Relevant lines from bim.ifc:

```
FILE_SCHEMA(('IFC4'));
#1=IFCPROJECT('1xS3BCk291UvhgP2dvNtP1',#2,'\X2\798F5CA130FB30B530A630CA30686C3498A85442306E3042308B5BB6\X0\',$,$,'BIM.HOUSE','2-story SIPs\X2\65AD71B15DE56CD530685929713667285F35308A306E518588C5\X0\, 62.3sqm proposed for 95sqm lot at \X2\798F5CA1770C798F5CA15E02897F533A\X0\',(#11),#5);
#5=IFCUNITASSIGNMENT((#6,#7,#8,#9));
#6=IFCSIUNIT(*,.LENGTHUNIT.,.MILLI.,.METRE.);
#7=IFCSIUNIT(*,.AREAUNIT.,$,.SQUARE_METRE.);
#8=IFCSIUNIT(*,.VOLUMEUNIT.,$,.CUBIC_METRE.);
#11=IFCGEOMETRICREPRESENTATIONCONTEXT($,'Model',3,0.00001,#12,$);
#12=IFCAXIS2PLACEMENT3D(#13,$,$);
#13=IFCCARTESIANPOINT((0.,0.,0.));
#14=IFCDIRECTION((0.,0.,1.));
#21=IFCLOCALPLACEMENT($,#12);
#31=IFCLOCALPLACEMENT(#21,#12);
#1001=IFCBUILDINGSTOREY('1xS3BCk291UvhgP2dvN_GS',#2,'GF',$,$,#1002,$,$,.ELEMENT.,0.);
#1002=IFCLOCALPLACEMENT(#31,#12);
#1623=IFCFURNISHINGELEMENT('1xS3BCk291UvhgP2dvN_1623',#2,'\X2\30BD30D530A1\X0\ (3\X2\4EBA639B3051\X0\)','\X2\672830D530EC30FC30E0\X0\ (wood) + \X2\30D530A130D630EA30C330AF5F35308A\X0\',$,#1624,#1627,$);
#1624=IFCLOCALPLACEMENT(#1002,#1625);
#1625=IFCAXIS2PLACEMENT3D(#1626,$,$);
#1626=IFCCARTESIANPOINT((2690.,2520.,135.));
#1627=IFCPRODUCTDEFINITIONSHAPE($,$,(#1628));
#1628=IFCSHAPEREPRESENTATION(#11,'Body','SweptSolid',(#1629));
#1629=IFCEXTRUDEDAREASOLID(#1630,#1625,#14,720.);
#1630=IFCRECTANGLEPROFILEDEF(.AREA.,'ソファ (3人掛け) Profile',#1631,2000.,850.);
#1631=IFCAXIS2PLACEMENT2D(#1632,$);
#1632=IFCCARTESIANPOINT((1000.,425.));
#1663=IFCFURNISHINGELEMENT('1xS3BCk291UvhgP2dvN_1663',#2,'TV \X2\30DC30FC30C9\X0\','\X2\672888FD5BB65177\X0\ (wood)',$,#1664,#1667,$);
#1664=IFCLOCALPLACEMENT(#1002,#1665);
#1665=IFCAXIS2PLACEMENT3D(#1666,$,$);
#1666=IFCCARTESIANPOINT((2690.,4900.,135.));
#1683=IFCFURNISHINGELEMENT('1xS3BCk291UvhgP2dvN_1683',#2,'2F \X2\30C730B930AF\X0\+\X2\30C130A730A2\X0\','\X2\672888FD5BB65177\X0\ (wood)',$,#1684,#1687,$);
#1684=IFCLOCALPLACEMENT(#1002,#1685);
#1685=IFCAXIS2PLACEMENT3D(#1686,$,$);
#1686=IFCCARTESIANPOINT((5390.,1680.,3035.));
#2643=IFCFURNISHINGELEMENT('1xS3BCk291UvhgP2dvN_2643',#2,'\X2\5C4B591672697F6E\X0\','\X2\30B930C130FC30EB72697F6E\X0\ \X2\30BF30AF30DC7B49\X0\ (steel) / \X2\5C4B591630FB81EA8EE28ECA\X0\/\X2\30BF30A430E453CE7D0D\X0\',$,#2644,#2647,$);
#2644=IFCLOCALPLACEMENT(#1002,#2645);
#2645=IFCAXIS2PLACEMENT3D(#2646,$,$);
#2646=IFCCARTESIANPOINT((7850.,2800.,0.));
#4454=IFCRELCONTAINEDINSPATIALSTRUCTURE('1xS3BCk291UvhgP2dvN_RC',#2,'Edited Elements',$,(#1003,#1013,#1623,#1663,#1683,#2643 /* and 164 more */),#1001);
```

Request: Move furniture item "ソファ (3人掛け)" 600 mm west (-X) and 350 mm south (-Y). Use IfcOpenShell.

```python
import ifcopenshell
import ifcopenshell.api.geometry
import ifcopenshell.util.placement
import ifcopenshell.util.unit

model = ifcopenshell.open("bim.ifc")
unit_scale = ifcopenshell.util.unit.calculate_unit_scale(model)

item = model.by_guid("1xS3BCk291UvhgP2dvN_1623")
matrix = ifcopenshell.util.placement.get_local_placement(item.ObjectPlacement)
matrix[0, 3] -= 0.6 / unit_scale
matrix[1, 3] -= 0.35 / unit_scale
ifcopenshell.api.geometry.edit_object_placement(model, product=item, matrix=matrix, is_si=False)

print(ifcopenshell.util.placement.get_local_placement(item.ObjectPlacement).round(3) + 0.0)

model.write("bim_rev.ifc")
```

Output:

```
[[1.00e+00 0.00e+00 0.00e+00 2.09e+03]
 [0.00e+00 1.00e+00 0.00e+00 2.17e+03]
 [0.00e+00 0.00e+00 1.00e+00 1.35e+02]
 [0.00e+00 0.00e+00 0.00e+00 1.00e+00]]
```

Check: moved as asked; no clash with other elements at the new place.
